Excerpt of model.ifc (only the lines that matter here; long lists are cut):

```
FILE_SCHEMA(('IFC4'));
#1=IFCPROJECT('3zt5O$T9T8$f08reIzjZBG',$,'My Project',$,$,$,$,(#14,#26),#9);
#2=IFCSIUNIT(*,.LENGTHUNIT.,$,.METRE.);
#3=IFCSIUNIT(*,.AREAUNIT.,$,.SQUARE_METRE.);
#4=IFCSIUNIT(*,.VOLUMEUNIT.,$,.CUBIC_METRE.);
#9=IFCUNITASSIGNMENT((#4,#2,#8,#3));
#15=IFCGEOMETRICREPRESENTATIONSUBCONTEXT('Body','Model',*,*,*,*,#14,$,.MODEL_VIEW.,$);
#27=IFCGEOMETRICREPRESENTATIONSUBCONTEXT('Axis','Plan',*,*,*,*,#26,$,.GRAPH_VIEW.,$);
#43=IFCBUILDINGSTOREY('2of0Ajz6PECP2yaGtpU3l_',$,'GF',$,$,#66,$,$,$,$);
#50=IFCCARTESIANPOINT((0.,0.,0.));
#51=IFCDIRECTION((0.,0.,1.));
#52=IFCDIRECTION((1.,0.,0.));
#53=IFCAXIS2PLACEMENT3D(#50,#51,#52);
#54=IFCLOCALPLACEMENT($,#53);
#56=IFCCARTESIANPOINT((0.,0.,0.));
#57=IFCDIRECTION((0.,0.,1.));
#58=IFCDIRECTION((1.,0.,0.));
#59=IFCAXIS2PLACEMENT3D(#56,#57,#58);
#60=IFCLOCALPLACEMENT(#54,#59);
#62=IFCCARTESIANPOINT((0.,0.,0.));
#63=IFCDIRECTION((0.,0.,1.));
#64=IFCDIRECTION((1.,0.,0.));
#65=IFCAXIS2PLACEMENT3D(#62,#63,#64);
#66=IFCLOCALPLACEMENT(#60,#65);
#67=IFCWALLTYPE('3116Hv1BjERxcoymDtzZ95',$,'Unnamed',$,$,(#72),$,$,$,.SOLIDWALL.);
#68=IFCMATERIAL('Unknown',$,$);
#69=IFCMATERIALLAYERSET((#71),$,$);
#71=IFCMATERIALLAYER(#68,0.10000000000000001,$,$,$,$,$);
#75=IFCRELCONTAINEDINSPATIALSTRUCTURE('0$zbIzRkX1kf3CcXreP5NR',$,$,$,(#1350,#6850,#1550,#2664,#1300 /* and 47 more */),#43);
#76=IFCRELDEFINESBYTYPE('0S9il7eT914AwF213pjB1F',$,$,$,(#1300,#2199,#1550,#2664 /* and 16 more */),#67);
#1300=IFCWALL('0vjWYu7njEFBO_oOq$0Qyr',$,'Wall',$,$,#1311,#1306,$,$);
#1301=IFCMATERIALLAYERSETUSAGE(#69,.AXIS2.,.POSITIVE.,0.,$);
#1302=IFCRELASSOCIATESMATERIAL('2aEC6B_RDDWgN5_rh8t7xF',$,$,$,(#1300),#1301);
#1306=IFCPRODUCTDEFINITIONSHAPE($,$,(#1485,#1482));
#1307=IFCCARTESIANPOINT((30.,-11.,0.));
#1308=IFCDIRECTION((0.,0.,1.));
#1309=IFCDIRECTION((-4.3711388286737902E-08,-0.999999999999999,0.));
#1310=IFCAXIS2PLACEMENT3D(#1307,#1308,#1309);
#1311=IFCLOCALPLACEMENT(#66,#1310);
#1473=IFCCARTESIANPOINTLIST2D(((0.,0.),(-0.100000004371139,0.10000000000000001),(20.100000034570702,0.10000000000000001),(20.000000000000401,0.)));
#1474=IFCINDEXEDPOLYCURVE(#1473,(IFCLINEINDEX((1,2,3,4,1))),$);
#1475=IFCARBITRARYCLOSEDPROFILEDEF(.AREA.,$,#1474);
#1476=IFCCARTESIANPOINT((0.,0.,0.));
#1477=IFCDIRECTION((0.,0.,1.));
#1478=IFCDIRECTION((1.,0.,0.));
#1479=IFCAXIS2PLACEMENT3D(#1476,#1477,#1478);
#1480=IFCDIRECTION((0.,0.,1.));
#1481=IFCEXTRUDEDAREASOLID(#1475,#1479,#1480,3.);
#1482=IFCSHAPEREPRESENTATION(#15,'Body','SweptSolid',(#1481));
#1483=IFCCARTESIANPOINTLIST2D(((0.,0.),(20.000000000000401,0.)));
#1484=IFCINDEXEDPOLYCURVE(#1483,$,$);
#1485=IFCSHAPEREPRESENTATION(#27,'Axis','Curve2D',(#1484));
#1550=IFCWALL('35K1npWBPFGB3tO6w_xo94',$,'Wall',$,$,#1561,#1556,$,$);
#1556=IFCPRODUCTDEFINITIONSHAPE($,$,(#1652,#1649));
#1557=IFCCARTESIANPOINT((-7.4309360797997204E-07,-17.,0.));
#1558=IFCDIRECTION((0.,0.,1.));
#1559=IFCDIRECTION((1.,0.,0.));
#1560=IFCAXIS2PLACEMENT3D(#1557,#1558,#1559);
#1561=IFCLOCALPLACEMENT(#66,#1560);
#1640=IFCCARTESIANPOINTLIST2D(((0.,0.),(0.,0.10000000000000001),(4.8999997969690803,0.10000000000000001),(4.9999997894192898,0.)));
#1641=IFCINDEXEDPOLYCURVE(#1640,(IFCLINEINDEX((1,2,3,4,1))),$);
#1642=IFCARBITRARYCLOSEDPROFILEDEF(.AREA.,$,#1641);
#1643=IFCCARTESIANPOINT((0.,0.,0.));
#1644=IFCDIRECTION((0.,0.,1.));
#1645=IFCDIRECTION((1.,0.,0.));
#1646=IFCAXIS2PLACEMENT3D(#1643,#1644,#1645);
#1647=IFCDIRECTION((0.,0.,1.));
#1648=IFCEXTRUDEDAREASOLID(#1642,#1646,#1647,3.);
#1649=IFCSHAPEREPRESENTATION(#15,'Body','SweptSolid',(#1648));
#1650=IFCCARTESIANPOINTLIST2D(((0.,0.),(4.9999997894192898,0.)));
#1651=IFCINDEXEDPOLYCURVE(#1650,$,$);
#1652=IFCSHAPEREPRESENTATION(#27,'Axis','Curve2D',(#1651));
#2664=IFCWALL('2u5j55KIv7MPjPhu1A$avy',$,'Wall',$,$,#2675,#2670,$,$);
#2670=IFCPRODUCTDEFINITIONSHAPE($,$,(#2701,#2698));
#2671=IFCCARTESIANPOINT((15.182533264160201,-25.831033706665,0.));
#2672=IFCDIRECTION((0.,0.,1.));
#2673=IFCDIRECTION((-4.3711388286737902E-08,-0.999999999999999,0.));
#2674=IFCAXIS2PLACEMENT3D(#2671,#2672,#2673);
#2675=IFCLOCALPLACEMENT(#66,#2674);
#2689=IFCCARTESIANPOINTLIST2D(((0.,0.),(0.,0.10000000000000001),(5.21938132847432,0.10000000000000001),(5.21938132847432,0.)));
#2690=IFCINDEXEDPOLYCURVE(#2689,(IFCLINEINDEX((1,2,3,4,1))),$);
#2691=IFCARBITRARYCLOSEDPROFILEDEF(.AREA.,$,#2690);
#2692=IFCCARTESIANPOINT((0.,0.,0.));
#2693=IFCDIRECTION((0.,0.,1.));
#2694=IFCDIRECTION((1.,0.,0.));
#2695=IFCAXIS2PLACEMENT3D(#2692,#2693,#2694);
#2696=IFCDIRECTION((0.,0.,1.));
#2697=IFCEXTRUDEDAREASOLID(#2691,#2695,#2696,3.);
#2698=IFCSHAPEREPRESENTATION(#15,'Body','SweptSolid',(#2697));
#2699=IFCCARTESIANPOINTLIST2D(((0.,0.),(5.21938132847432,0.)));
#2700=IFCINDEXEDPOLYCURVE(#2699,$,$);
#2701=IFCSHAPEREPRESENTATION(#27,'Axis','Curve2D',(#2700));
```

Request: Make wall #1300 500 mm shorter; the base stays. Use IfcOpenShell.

```python
import ifcopenshell
import ifcopenshell.geom
import ifcopenshell.util.representation
import ifcopenshell.util.shape
import ifcopenshell.util.unit

model = ifcopenshell.open("model.ifc")
unit_scale = ifcopenshell.util.unit.calculate_unit_scale(model)
settings = ifcopenshell.geom.settings()


def volume(element):
    """Net volume in cubic metres, openings subtracted."""
    shape = ifcopenshell.geom.create_shape(settings, element)
    return ifcopenshell.util.shape.get_volume(shape.geometry)


wall = model.by_guid("0vjWYu7njEFBO_oOq$0Qyr")
before = volume(wall)

body = ifcopenshell.util.representation.get_representation(wall, "Model", "Body")
solid = body.Items[0]
old_height = solid.Depth
solid.Depth -= 0.5 / unit_scale
after = volume(wall)

print(f"height {old_height:g} -> {solid.Depth:g}, volume {before:.3f} -> {after:.3f} m3")

model.write("model_v2.ifc")
```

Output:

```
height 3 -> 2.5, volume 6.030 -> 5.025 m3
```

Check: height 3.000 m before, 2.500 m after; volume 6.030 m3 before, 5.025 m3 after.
